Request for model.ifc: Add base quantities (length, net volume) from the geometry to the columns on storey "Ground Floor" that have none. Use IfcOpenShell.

First a look at what the model holds.

```python
import ifcopenshell
import ifcopenshell.util.element
import ifcopenshell.util.unit

model = ifcopenshell.open("model.ifc")
print(model.schema)
for unit_type in ("LENGTHUNIT", "AREAUNIT", "VOLUMEUNIT"):
    print(unit_type, ifcopenshell.util.unit.calculate_unit_scale(model, unit_type))
storey = next(s for s in model.by_type("IfcBuildingStorey") if s.Name == "Ground Floor")
columns = [e for e in ifcopenshell.util.element.get_decomposition(storey) if e.is_a("IfcColumn")]
for e in sorted(columns, key=lambda e: e.id()):
    print(e.id(), e.is_a(), e.Name, list(ifcopenshell.util.element.get_psets(e, qtos_only=True)), sep=" | ")
```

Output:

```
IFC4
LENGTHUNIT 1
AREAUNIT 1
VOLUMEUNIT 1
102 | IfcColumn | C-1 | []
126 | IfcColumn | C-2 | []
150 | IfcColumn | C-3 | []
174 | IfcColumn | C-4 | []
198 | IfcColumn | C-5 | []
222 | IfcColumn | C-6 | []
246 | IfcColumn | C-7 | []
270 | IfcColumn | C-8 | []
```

```python
import ifcopenshell
import ifcopenshell.api.pset
import ifcopenshell.geom
import ifcopenshell.util.element
import ifcopenshell.util.shape
import ifcopenshell.util.unit

model = ifcopenshell.open("model.ifc")
unit_scale = ifcopenshell.util.unit.calculate_unit_scale(model)
volume_scale = ifcopenshell.util.unit.calculate_unit_scale(model, "VOLUMEUNIT")
settings = ifcopenshell.geom.settings()

storey = next(s for s in model.by_type("IfcBuildingStorey") if s.Name == "Ground Floor")
columns = [e for e in ifcopenshell.util.element.get_decomposition(storey) if e.is_a("IfcColumn")]

for e in sorted(columns, key=lambda e: e.id()):
    if ifcopenshell.util.element.get_psets(e, qtos_only=True, should_inherit=False):
        continue
    # Geometry comes back in metres, in the element's own axes.
    shape = ifcopenshell.geom.create_shape(settings, e)
    values = {
        "Length": ifcopenshell.util.shape.get_z(shape.geometry) / unit_scale,
        "NetVolume": ifcopenshell.util.shape.get_volume(shape.geometry) / volume_scale,
    }
    qto = ifcopenshell.api.pset.add_qto(model, product=e, name="Qto_ColumnBaseQuantities")
    ifcopenshell.api.pset.edit_qto(model, qto=qto, properties=values)
    print(e.id(), {k: round(v, 3) for k, v in values.items()})

model.write("model-out.ifc")
```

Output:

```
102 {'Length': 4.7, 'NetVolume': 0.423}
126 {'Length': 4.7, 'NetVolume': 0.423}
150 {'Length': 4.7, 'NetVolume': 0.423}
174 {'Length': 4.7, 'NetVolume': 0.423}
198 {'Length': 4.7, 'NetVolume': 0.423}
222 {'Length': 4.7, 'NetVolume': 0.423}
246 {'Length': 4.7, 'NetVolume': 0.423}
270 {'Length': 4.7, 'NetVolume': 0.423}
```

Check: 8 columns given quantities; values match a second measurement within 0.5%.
